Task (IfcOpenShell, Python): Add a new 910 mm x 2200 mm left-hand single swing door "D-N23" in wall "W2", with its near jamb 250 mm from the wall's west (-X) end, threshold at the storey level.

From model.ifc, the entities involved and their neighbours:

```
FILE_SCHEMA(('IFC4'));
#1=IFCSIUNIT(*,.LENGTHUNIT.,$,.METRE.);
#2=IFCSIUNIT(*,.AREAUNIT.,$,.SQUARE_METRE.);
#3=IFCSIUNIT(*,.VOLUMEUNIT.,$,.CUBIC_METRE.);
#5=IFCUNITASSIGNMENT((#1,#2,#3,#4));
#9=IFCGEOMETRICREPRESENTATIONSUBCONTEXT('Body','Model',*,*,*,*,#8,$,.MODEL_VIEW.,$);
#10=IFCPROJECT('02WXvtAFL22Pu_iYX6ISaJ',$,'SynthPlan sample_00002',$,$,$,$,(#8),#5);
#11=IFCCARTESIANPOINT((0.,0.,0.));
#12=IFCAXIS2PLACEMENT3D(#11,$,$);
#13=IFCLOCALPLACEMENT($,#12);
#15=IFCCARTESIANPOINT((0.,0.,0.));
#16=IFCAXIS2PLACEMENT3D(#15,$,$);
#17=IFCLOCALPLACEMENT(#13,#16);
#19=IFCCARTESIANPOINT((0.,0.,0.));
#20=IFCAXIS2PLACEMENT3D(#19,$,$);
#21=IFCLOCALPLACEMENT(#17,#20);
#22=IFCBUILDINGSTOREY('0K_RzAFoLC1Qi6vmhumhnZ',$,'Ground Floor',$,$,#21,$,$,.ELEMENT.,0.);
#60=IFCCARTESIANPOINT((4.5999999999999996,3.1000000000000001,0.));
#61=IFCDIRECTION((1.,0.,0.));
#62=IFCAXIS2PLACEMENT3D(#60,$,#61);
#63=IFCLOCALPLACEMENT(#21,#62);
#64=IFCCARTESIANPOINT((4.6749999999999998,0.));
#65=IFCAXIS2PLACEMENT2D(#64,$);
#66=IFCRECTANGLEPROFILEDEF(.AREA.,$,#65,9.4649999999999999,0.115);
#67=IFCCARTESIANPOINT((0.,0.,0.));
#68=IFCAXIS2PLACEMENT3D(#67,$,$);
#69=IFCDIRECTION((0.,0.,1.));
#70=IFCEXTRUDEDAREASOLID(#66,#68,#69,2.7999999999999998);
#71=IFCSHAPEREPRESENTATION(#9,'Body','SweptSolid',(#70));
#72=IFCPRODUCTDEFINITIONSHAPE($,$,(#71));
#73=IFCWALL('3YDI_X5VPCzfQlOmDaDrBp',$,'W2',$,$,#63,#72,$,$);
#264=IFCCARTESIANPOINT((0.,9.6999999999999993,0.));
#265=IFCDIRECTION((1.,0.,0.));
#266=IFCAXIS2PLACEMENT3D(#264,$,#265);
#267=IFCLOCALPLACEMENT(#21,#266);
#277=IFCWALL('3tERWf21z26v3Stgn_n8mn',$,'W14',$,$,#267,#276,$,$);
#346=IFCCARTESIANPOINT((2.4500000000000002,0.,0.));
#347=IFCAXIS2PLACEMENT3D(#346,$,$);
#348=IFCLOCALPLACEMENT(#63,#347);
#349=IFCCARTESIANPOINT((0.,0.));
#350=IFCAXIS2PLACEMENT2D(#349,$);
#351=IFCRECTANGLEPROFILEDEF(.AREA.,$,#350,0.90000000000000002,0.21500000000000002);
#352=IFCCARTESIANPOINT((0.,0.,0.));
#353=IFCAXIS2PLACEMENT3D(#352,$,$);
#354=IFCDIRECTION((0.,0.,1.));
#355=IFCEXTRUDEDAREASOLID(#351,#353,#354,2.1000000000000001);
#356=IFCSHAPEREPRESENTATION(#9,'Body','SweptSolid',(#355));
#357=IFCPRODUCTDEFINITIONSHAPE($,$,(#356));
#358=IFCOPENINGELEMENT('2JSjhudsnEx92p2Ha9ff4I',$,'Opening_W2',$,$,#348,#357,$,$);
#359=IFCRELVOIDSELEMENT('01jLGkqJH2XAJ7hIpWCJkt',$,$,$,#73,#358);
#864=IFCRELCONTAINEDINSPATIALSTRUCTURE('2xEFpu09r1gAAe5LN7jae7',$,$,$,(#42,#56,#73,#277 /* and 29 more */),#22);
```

```python
import numpy as np
import ifcopenshell
import ifcopenshell.api.feature
import ifcopenshell.api.geometry
import ifcopenshell.api.root
import ifcopenshell.api.spatial
import ifcopenshell.geom
import ifcopenshell.util.element
import ifcopenshell.util.placement
import ifcopenshell.util.representation
import ifcopenshell.util.shape
import ifcopenshell.util.unit

model = ifcopenshell.open("model.ifc")
unit_scale = ifcopenshell.util.unit.calculate_unit_scale(model)
settings = ifcopenshell.geom.settings()


def volume(element):
    """Net volume in cubic metres, openings subtracted."""
    shape = ifcopenshell.geom.create_shape(settings, element)
    return ifcopenshell.util.shape.get_volume(shape.geometry)


wall = model.by_guid("3YDI_X5VPCzfQlOmDaDrBp")
storey = ifcopenshell.util.element.get_container(wall, ifc_class="IfcBuildingStorey")
context = ifcopenshell.util.representation.get_context(model, "Model", "Body", "MODEL_VIEW")
before = volume(wall)

width, height, from_end, sill = 0.91, 2.2, 0.25, 0.0  # metres

# The wall runs along its own X axis, and the end named is its -X end.
wall_shape = ifcopenshell.geom.create_shape(settings, wall)
x, y, z = ifcopenshell.util.shape.get_vertices(wall_shape.geometry).T
start = x.min() + from_end
face, thickness = float(y.min()), float(y.max() - y.min())
wall_matrix = ifcopenshell.util.placement.get_local_placement(wall.ObjectPlacement)
level = ifcopenshell.util.placement.get_local_placement(storey.ObjectPlacement)[2, 3]


def in_wall(x, y):
    """Placement at x, y metres in the wall's axes, at sill height."""
    matrix = wall_matrix.copy()
    matrix[:, 3] = wall_matrix @ np.array([x / unit_scale, y / unit_scale, 0.0, 1.0])
    matrix[2, 3] = level + sill / unit_scale
    return matrix


# Opening: a box that overshoots both wall faces by 50 mm.
opening = ifcopenshell.api.root.create_entity(model, ifc_class="IfcOpeningElement", predefined_type="OPENING")
box = ifcopenshell.api.geometry.add_wall_representation(
    model, context=context, length=width, height=height, thickness=thickness + 0.1
)
ifcopenshell.api.geometry.assign_representation(model, product=opening, representation=box)
ifcopenshell.api.geometry.edit_object_placement(model, product=opening, matrix=in_wall(start, face - 0.05), is_si=False)
ifcopenshell.api.feature.add_feature(model, feature=opening, element=wall)

door = ifcopenshell.api.root.create_entity(model, ifc_class="IfcDoor", name="D-N23", predefined_type="DOOR")
door.OverallWidth, door.OverallHeight = width / unit_scale, height / unit_scale
door.OperationType = "SINGLE_SWING_LEFT"
body = ifcopenshell.api.geometry.add_door_representation(
    model,
    context=context,
    overall_width=door.OverallWidth,
    overall_height=door.OverallHeight,
    operation_type="SINGLE_SWING_LEFT",
    lining_properties={"LiningDepth": thickness / unit_scale, "ThresholdDepth": thickness / unit_scale},
)
ifcopenshell.api.geometry.assign_representation(model, product=door, representation=body)
ifcopenshell.api.spatial.assign_container(model, products=[door], relating_structure=storey)
ifcopenshell.api.feature.add_filling(model, opening=opening, element=door)

# The lining spans the wall, so the door starts at the wall face.
ifcopenshell.api.geometry.edit_object_placement(model, product=door, matrix=in_wall(start, face), is_si=False)

after = volume(wall)

print(f"wall volume {before:.3f} -> {after:.3f} m3")

model.write("model-out.ifc")
```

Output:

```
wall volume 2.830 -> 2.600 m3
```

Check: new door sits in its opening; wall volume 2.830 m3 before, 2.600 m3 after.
